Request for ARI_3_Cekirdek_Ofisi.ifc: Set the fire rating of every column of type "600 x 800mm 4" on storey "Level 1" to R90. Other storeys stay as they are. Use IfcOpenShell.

First a look at what the model holds.

```python
import ifcopenshell
import ifcopenshell.util.element

model = ifcopenshell.open("ARI_3_Cekirdek_Ofisi.ifc")
print(model.schema)
storey = next(s for s in model.by_type("IfcBuildingStorey") if s.Name == "Level 1")
columns = [e for e in ifcopenshell.util.element.get_decomposition(storey) if e.is_a("IfcColumn")]
seen = {}
for e in columns:
    element_type = ifcopenshell.util.element.get_type(e)
    key = (element_type.Name if element_type != e and element_type else None, ifcopenshell.util.element.get_pset(e, "Pset_ColumnCommon", "FireRating"))
    seen[key] = seen.get(key, 0) + 1
for (name, value), count in sorted(seen.items(), key=str):
    print(count, "x", name, "|", value)
```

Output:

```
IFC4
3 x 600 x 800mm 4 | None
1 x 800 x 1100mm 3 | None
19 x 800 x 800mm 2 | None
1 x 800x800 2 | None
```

```python
import ifcopenshell
import ifcopenshell.api.pset
import ifcopenshell.util.element

model = ifcopenshell.open("ARI_3_Cekirdek_Ofisi.ifc")

storey = next(s for s in model.by_type("IfcBuildingStorey") if s.Name == "Level 1")
columns = [e for e in ifcopenshell.util.element.get_decomposition(storey) if e.is_a("IfcColumn")]

count = 0
for e in columns:
    element_type = ifcopenshell.util.element.get_type(e)
    if element_type in (None, e) or element_type.Name != "600 x 800mm 4":
        continue
    # add_pset returns the element's existing set when there is one.
    pset = ifcopenshell.api.pset.add_pset(model, product=e, name="Pset_ColumnCommon")
    ifcopenshell.api.pset.edit_pset(model, pset=pset, properties={"FireRating": "R90"})
    count += 1

print(count, "columns updated")

model.write("ARI_3_Cekirdek_Ofisi_edited.ifc")
```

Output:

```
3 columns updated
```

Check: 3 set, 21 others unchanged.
